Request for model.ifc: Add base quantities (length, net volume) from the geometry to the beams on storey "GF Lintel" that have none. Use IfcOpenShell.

First a look at what the model holds.

```python
import ifcopenshell
import ifcopenshell.util.element
import ifcopenshell.util.unit

model = ifcopenshell.open("model.ifc")
print(model.schema)
for unit_type in ("LENGTHUNIT", "AREAUNIT", "VOLUMEUNIT"):
    print(unit_type, ifcopenshell.util.unit.calculate_unit_scale(model, unit_type))
storey = next(s for s in model.by_type("IfcBuildingStorey") if s.Name == "GF Lintel")
beams = [e for e in ifcopenshell.util.element.get_decomposition(storey) if e.is_a("IfcBeam")]
for e in sorted(beams, key=lambda e: e.id()):
    print(e.id(), e.is_a(), e.Name, list(ifcopenshell.util.element.get_psets(e, qtos_only=True)), sep=" | ")
```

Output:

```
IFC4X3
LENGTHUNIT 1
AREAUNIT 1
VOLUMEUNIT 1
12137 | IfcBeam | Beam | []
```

```python
import ifcopenshell
import ifcopenshell.api.pset
import ifcopenshell.geom
import ifcopenshell.util.element
import ifcopenshell.util.shape
import ifcopenshell.util.unit

model = ifcopenshell.open("model.ifc")
unit_scale = ifcopenshell.util.unit.calculate_unit_scale(model)
volume_scale = ifcopenshell.util.unit.calculate_unit_scale(model, "VOLUMEUNIT")
settings = ifcopenshell.geom.settings()

storey = next(s for s in model.by_type("IfcBuildingStorey") if s.Name == "GF Lintel")
beams = [e for e in ifcopenshell.util.element.get_decomposition(storey) if e.is_a("IfcBeam")]

for e in sorted(beams, key=lambda e: e.id()):
    if ifcopenshell.util.element.get_psets(e, qtos_only=True, should_inherit=False):
        continue
    # Geometry comes back in metres, in the element's own axes.
    shape = ifcopenshell.geom.create_shape(settings, e)
    values = {
        "Length": ifcopenshell.util.shape.get_max_xyz(shape.geometry) / unit_scale,
        "NetVolume": ifcopenshell.util.shape.get_volume(shape.geometry) / volume_scale,
    }
    qto = ifcopenshell.api.pset.add_qto(model, product=e, name="Qto_BeamBaseQuantities")
    ifcopenshell.api.pset.edit_qto(model, qto=qto, properties=values)
    print(e.id(), {k: round(v, 3) for k, v in values.items()})

model.write("model_updated.ifc")
```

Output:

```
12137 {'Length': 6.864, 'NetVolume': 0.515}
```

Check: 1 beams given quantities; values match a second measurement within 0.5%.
